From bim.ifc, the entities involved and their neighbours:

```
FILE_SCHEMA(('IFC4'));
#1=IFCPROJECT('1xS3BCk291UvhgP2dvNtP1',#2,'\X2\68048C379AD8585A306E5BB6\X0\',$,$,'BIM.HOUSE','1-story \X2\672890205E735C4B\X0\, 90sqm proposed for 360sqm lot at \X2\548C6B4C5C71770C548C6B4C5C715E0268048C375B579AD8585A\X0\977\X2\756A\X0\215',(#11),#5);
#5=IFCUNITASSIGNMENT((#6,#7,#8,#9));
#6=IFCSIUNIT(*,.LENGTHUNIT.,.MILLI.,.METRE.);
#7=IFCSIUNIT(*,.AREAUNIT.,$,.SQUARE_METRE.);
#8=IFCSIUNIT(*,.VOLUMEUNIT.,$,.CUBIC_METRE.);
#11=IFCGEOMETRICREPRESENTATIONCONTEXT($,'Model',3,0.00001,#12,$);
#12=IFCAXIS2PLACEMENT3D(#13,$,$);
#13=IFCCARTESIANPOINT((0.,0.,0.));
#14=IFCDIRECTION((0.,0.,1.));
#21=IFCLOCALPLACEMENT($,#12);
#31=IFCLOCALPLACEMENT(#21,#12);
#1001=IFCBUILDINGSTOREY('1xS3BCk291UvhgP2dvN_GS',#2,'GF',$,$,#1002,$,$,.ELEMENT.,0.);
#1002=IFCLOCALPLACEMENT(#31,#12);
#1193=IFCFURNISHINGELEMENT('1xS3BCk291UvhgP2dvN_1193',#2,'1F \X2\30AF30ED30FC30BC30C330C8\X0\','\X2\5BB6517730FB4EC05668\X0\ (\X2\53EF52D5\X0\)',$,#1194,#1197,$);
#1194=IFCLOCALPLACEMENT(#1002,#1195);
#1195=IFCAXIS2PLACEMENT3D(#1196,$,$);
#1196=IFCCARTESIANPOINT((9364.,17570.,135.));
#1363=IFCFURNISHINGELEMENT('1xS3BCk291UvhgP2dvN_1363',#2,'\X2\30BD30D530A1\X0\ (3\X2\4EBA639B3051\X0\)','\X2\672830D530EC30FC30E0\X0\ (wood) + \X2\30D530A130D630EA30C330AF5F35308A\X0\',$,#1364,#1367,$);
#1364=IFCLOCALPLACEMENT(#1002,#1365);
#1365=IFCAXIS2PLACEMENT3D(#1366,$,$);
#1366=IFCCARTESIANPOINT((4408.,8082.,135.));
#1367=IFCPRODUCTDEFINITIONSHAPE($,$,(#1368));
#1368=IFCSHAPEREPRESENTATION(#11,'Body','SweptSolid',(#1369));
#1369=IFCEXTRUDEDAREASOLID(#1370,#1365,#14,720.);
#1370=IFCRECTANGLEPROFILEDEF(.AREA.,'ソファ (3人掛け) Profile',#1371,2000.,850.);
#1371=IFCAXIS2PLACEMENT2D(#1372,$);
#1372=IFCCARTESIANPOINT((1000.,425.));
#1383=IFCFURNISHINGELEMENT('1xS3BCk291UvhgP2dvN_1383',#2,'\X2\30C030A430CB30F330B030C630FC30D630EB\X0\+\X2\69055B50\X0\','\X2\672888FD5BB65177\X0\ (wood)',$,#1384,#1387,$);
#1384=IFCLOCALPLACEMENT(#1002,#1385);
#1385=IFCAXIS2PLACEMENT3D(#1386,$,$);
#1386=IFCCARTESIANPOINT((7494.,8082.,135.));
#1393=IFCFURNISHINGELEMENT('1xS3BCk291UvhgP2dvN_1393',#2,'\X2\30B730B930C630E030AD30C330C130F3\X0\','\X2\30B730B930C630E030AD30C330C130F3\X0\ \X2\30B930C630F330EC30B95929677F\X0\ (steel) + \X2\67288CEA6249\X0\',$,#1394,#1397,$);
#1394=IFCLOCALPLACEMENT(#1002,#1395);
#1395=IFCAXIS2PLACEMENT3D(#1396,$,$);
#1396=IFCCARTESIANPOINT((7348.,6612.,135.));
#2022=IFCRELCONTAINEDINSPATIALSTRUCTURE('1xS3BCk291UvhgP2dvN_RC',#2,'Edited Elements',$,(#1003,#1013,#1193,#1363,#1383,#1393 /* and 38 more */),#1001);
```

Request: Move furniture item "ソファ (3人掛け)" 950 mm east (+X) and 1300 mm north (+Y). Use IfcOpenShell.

```python
import ifcopenshell
import ifcopenshell.api.geometry
import ifcopenshell.util.placement
import ifcopenshell.util.unit

model = ifcopenshell.open("bim.ifc")
unit_scale = ifcopenshell.util.unit.calculate_unit_scale(model)

item = model.by_guid("1xS3BCk291UvhgP2dvN_1363")
matrix = ifcopenshell.util.placement.get_local_placement(item.ObjectPlacement)
matrix[0, 3] += 0.95 / unit_scale
matrix[1, 3] += 1.3 / unit_scale
ifcopenshell.api.geometry.edit_object_placement(model, product=item, matrix=matrix, is_si=False)

print(ifcopenshell.util.placement.get_local_placement(item.ObjectPlacement).round(3) + 0.0)

model.write("bim_rev.ifc")
```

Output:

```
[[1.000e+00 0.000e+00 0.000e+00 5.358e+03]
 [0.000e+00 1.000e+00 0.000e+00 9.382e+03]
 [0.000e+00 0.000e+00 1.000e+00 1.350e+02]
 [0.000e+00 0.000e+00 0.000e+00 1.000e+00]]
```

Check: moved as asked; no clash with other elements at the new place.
